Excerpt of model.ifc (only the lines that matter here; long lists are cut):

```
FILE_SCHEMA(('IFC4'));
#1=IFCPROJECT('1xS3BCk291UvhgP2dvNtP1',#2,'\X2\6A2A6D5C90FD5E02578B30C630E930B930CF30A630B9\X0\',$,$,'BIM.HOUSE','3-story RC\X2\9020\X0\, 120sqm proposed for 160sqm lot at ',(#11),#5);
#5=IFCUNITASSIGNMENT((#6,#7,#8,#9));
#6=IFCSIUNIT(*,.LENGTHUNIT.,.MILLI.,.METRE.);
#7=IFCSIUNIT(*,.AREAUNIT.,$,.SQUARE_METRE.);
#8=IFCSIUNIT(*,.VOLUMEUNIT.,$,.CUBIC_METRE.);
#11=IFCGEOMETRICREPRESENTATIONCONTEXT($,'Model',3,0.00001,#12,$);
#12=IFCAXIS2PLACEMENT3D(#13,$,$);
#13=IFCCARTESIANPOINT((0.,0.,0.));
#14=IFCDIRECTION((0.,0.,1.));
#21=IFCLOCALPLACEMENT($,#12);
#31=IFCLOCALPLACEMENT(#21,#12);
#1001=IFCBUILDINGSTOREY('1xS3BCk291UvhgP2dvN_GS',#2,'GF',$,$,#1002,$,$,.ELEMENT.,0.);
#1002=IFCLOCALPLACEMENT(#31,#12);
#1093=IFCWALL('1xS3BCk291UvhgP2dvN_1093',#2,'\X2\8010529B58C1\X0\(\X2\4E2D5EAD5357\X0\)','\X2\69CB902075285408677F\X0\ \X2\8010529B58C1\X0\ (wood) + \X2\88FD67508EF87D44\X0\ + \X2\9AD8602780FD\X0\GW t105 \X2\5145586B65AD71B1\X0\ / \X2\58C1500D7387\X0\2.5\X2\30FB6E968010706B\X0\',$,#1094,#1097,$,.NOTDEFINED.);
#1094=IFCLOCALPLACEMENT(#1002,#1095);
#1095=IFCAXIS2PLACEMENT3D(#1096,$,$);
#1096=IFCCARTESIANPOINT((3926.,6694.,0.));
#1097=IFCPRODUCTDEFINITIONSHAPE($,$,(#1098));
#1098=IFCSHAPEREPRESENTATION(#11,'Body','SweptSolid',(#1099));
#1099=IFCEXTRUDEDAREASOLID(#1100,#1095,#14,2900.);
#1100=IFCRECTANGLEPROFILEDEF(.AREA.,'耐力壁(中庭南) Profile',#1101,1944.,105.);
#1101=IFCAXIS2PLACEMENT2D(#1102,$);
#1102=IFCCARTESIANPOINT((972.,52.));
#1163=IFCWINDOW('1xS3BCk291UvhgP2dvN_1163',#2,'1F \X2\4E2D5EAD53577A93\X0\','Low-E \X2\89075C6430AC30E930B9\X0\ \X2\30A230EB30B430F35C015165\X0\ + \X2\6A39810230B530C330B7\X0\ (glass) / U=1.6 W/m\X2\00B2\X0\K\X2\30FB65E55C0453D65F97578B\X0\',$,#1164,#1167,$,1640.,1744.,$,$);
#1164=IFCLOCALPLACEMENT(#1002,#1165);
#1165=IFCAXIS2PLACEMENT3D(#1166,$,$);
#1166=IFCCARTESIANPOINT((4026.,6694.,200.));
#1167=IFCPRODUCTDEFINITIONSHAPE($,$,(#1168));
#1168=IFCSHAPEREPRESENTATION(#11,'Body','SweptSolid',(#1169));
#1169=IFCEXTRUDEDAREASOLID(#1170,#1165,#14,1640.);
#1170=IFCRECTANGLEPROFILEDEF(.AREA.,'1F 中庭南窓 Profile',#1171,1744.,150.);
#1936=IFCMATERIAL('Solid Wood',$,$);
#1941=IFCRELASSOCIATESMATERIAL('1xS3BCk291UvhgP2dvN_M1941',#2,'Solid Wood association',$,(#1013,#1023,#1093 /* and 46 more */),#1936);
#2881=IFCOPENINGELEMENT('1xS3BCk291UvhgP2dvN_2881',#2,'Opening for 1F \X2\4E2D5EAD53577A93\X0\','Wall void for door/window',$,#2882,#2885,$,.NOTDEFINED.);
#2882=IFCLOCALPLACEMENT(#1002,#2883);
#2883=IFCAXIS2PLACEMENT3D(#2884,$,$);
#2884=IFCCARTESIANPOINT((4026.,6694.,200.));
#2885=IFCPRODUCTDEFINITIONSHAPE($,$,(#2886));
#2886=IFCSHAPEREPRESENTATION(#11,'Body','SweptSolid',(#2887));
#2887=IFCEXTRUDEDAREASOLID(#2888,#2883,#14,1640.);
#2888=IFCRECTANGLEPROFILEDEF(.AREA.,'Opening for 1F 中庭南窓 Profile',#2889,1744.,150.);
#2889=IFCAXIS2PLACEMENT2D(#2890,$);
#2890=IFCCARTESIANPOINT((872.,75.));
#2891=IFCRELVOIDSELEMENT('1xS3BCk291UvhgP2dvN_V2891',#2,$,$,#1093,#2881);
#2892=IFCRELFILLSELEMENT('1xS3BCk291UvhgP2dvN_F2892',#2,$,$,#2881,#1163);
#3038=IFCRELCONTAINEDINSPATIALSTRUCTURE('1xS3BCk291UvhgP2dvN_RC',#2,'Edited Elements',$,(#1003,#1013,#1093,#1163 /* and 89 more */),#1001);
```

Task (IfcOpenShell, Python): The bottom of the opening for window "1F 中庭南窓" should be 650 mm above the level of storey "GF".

```python
import numpy as np
import ifcopenshell
import ifcopenshell.api.geometry
import ifcopenshell.geom
import ifcopenshell.util.element
import ifcopenshell.util.placement
import ifcopenshell.util.shape
import ifcopenshell.util.unit

model = ifcopenshell.open("model.ifc")
unit_scale = ifcopenshell.util.unit.calculate_unit_scale(model)

window = model.by_guid("1xS3BCk291UvhgP2dvN_1163")
opening = window.FillsVoids[0].RelatingOpeningElement
storey = ifcopenshell.util.element.get_container(window, ifc_class="IfcBuildingStorey")
level = ifcopenshell.util.placement.get_local_placement(storey.ObjectPlacement)[2, 3]

# The opening's origin need not be at the sill, so measure its lowest point.
shape = ifcopenshell.geom.create_shape(ifcopenshell.geom.settings(), opening)
bottom = ifcopenshell.util.shape.get_shape_bottom_elevation(shape, shape.geometry) / unit_scale
dz = level + 650.0 - bottom

shift = np.array([0.0, 0.0, dz])
# The window is not placed relative to its opening, so move both.
for product in (opening, window):
    matrix = ifcopenshell.util.placement.get_local_placement(product.ObjectPlacement)
    matrix[:3, 3] += shift
    ifcopenshell.api.geometry.edit_object_placement(model, product=product, matrix=matrix, is_si=False)

print(f"moved by {dz * unit_scale:+.3f} m")

model.write("model-out.ifc")
```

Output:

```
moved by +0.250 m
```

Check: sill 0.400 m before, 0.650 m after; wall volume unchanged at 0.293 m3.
